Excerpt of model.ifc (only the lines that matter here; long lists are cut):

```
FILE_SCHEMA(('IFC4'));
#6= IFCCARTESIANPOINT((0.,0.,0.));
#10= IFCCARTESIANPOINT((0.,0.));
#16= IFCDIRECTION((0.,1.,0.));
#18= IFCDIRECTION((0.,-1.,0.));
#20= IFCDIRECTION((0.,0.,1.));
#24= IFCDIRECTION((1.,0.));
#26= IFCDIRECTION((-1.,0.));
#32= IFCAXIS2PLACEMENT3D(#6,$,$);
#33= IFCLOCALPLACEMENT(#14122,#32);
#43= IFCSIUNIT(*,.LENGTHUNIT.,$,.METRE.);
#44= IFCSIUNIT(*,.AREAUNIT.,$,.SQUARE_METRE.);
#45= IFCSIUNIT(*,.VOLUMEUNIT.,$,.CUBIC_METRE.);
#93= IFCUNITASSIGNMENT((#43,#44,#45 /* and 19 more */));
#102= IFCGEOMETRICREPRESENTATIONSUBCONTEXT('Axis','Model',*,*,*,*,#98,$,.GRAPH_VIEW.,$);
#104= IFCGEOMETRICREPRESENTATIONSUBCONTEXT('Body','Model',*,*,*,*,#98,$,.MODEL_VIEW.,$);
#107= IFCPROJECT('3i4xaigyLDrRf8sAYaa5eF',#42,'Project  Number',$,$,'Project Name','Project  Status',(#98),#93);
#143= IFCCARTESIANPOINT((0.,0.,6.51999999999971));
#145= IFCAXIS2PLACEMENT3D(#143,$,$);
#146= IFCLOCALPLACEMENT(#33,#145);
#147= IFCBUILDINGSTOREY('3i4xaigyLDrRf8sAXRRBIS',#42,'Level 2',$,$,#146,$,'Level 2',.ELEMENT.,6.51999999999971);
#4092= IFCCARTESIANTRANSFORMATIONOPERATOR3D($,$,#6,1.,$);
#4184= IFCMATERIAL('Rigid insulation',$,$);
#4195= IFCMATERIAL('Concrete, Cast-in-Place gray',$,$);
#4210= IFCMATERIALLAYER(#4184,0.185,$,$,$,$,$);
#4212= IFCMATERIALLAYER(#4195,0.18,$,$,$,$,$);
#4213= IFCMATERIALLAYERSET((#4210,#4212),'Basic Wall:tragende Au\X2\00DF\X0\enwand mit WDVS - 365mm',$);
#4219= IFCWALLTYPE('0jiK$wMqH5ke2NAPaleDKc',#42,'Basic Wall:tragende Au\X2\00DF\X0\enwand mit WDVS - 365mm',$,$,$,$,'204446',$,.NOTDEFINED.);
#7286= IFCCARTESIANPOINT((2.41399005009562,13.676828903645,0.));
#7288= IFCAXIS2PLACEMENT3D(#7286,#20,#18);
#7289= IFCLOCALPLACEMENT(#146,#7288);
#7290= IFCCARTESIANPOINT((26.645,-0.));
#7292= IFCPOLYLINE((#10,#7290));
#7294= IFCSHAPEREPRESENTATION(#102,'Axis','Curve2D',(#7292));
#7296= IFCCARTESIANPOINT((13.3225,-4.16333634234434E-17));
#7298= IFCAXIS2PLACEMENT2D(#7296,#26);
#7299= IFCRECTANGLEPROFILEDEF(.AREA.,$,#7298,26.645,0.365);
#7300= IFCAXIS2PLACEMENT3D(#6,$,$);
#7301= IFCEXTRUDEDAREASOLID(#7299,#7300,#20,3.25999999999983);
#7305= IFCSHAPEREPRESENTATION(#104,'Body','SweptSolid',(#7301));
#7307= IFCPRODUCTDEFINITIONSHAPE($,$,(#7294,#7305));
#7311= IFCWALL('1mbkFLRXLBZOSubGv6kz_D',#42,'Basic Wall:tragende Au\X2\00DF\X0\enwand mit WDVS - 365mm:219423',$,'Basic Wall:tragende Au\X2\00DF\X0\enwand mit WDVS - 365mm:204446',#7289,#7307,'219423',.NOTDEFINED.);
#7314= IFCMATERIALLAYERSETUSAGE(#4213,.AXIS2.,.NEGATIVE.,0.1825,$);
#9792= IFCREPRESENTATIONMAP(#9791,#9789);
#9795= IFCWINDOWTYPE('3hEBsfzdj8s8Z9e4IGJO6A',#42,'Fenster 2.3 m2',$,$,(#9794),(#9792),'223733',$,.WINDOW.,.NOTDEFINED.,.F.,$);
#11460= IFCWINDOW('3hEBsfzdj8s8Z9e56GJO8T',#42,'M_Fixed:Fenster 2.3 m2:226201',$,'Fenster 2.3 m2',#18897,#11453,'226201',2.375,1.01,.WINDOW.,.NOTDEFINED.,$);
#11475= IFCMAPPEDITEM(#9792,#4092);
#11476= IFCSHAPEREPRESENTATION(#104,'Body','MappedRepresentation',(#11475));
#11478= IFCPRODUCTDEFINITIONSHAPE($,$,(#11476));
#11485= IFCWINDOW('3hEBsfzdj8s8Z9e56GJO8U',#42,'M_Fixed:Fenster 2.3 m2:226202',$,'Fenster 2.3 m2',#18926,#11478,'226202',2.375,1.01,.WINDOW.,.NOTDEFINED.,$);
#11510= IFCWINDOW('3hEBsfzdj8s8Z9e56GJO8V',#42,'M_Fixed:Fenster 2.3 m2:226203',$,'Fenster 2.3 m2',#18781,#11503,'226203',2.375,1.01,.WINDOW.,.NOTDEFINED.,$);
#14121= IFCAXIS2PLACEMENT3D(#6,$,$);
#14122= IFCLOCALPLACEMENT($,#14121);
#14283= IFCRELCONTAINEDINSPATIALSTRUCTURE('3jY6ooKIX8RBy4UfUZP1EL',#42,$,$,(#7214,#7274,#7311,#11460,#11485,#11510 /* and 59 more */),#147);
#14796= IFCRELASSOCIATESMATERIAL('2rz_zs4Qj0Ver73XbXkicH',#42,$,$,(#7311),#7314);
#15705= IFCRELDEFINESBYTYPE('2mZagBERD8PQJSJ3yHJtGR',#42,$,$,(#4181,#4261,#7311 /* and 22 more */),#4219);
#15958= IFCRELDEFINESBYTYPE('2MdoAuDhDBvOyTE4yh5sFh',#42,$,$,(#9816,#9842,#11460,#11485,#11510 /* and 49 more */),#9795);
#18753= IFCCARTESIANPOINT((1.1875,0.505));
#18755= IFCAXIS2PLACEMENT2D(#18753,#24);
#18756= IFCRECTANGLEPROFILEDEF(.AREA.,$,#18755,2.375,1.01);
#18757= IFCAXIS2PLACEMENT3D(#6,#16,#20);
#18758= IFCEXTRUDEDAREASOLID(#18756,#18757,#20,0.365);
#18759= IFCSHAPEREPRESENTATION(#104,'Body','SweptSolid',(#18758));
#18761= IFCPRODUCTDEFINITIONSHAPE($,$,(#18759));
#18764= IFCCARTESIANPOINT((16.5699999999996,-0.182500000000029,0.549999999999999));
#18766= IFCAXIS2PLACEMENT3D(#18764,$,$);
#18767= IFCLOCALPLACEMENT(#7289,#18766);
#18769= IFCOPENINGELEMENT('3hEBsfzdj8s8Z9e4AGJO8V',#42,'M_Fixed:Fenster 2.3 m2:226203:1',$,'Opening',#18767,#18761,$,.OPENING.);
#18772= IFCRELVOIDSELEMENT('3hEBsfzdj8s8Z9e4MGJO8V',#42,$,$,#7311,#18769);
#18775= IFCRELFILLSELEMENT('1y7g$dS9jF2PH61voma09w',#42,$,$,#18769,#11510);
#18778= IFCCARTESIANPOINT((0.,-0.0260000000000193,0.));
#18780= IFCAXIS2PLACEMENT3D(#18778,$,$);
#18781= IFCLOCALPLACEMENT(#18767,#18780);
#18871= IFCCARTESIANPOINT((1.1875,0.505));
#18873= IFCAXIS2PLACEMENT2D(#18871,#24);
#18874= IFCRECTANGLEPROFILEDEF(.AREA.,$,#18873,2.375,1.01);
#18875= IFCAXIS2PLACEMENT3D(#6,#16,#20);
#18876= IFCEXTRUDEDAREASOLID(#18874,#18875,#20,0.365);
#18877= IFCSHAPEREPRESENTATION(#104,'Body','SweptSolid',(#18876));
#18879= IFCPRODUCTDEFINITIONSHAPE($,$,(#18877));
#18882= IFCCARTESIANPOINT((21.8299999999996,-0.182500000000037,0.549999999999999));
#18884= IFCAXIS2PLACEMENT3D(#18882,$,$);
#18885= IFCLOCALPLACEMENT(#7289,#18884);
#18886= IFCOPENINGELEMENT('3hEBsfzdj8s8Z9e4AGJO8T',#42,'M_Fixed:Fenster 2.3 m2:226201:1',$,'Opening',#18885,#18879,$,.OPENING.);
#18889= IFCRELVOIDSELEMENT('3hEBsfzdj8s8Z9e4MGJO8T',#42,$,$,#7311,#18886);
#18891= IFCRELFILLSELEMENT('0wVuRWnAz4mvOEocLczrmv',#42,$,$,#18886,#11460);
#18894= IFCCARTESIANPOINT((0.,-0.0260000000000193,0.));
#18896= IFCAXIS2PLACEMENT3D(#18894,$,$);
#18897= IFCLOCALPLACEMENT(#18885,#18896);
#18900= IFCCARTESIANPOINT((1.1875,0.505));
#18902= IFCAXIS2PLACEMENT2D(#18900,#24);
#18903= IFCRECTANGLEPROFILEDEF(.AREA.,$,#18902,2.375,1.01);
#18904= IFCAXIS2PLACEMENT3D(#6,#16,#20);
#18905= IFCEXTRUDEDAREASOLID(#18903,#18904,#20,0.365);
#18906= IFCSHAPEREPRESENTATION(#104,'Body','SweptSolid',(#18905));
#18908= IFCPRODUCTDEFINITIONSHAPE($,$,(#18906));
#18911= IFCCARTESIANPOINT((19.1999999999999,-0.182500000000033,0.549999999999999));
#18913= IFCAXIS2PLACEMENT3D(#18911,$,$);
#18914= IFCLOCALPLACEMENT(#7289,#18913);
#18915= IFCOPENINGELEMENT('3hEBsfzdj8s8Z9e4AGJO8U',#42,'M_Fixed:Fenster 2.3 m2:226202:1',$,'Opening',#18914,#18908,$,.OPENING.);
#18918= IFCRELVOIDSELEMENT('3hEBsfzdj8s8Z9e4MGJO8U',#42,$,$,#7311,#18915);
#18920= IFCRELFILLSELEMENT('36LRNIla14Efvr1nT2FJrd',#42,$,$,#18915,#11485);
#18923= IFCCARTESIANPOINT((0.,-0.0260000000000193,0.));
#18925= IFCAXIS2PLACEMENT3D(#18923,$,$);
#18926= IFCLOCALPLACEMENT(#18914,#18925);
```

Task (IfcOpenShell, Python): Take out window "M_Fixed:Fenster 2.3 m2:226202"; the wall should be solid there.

```python
import ifcopenshell
import ifcopenshell.api.feature
import ifcopenshell.api.root
import ifcopenshell.geom
import ifcopenshell.util.shape

model = ifcopenshell.open("model.ifc")
settings = ifcopenshell.geom.settings()


def volume(element):
    """Net volume in cubic metres, openings subtracted."""
    shape = ifcopenshell.geom.create_shape(settings, element)
    return ifcopenshell.util.shape.get_volume(shape.geometry)


window = model.by_id(11485)
opening = window.FillsVoids[0].RelatingOpeningElement
wall = opening.VoidsElements[0].RelatingBuildingElement
before = volume(wall)

ifcopenshell.api.root.remove_product(model, product=window)
ifcopenshell.api.feature.remove_feature(model, feature=opening)

after = volume(wall)

print(f"wall volume {before:.3f} -> {after:.3f} m3")

model.write("model_v2.ifc")
```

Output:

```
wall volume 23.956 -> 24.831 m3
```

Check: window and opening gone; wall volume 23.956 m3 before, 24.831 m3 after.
